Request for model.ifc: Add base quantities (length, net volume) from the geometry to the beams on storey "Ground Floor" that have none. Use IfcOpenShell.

First a look at what the model holds.

```python
import ifcopenshell
import ifcopenshell.util.element
import ifcopenshell.util.unit

model = ifcopenshell.open("model.ifc")
print(model.schema)
for unit_type in ("LENGTHUNIT", "AREAUNIT", "VOLUMEUNIT"):
    print(unit_type, ifcopenshell.util.unit.calculate_unit_scale(model, unit_type))
storey = next(s for s in model.by_type("IfcBuildingStorey") if s.Name == "Ground Floor")
beams = [e for e in ifcopenshell.util.element.get_decomposition(storey) if e.is_a("IfcBeam")]
for e in sorted(beams, key=lambda e: e.id()):
    print(e.id(), e.is_a(), e.Name, list(ifcopenshell.util.element.get_psets(e, qtos_only=True)), sep=" | ")
```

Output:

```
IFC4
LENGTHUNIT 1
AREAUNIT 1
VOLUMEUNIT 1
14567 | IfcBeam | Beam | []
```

```python
import ifcopenshell
import ifcopenshell.api.pset
import ifcopenshell.geom
import ifcopenshell.util.element
import ifcopenshell.util.shape
import ifcopenshell.util.unit

model = ifcopenshell.open("model.ifc")
unit_scale = ifcopenshell.util.unit.calculate_unit_scale(model)
volume_scale = ifcopenshell.util.unit.calculate_unit_scale(model, "VOLUMEUNIT")
settings = ifcopenshell.geom.settings()

storey = next(s for s in model.by_type("IfcBuildingStorey") if s.Name == "Ground Floor")
beams = [e for e in ifcopenshell.util.element.get_decomposition(storey) if e.is_a("IfcBeam")]

for e in sorted(beams, key=lambda e: e.id()):
    if ifcopenshell.util.element.get_psets(e, qtos_only=True, should_inherit=False):
        continue
    # Geometry comes back in metres, in the element's own axes.
    shape = ifcopenshell.geom.create_shape(settings, e)
    values = {
        "Length": ifcopenshell.util.shape.get_max_xyz(shape.geometry) / unit_scale,
        "NetVolume": ifcopenshell.util.shape.get_volume(shape.geometry) / volume_scale,
    }
    qto = ifcopenshell.api.pset.add_qto(model, product=e, name="Qto_BeamBaseQuantities")
    ifcopenshell.api.pset.edit_qto(model, qto=qto, properties=values)
    print(e.id(), {k: round(v, 3) for k, v in values.items()})

model.write("model_updated.ifc")
```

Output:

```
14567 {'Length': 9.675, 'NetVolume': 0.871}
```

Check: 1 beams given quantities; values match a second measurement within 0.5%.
